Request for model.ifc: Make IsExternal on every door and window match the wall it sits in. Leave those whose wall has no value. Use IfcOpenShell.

First a look at what the model holds.

```python
import ifcopenshell
import ifcopenshell.util.element

model = ifcopenshell.open("model.ifc")
print(model.schema)
seen = {}
for e in model.by_type("IfcDoor") + model.by_type("IfcWindow"):
    if not e.FillsVoids:
        continue
    host = e.FillsVoids[0].RelatingOpeningElement.VoidsElements[0].RelatingBuildingElement
    own = ifcopenshell.util.element.get_pset(e, f"Pset_{e.is_a()[3:].removesuffix('StandardCase')}Common", "IsExternal")
    wall = ifcopenshell.util.element.get_pset(host, "Pset_WallCommon", "IsExternal")
    seen[e.is_a(), own, wall] = seen.get((e.is_a(), own, wall), 0) + 1
for (cls, own, wall), count in sorted(seen.items(), key=str):
    print(count, cls, "IsExternal:", own, "| host wall:", wall)
```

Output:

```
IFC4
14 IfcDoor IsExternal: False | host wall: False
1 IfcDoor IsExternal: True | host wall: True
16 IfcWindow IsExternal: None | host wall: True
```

```python
import ifcopenshell
import ifcopenshell.api.pset
import ifcopenshell.util.element

model = ifcopenshell.open("model.ifc")

count = 0
for ifc_class, pset_name in (("IfcDoor", "Pset_DoorCommon"), ("IfcWindow", "Pset_WindowCommon")):
    for e in model.by_type(ifc_class):
        if not e.FillsVoids:
            continue
        host = e.FillsVoids[0].RelatingOpeningElement.VoidsElements[0].RelatingBuildingElement
        external = ifcopenshell.util.element.get_pset(host, "Pset_WallCommon", "IsExternal")
        if external is None or ifcopenshell.util.element.get_pset(e, pset_name, "IsExternal") == external:
            continue
        pset = ifcopenshell.api.pset.add_pset(model, product=e, name=pset_name)
        ifcopenshell.api.pset.edit_pset(model, pset=pset, properties={"IsExternal": external})
        count += 1

print(count, "updated")

model.write("model_v2.ifc")
```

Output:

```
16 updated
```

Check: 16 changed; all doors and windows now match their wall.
